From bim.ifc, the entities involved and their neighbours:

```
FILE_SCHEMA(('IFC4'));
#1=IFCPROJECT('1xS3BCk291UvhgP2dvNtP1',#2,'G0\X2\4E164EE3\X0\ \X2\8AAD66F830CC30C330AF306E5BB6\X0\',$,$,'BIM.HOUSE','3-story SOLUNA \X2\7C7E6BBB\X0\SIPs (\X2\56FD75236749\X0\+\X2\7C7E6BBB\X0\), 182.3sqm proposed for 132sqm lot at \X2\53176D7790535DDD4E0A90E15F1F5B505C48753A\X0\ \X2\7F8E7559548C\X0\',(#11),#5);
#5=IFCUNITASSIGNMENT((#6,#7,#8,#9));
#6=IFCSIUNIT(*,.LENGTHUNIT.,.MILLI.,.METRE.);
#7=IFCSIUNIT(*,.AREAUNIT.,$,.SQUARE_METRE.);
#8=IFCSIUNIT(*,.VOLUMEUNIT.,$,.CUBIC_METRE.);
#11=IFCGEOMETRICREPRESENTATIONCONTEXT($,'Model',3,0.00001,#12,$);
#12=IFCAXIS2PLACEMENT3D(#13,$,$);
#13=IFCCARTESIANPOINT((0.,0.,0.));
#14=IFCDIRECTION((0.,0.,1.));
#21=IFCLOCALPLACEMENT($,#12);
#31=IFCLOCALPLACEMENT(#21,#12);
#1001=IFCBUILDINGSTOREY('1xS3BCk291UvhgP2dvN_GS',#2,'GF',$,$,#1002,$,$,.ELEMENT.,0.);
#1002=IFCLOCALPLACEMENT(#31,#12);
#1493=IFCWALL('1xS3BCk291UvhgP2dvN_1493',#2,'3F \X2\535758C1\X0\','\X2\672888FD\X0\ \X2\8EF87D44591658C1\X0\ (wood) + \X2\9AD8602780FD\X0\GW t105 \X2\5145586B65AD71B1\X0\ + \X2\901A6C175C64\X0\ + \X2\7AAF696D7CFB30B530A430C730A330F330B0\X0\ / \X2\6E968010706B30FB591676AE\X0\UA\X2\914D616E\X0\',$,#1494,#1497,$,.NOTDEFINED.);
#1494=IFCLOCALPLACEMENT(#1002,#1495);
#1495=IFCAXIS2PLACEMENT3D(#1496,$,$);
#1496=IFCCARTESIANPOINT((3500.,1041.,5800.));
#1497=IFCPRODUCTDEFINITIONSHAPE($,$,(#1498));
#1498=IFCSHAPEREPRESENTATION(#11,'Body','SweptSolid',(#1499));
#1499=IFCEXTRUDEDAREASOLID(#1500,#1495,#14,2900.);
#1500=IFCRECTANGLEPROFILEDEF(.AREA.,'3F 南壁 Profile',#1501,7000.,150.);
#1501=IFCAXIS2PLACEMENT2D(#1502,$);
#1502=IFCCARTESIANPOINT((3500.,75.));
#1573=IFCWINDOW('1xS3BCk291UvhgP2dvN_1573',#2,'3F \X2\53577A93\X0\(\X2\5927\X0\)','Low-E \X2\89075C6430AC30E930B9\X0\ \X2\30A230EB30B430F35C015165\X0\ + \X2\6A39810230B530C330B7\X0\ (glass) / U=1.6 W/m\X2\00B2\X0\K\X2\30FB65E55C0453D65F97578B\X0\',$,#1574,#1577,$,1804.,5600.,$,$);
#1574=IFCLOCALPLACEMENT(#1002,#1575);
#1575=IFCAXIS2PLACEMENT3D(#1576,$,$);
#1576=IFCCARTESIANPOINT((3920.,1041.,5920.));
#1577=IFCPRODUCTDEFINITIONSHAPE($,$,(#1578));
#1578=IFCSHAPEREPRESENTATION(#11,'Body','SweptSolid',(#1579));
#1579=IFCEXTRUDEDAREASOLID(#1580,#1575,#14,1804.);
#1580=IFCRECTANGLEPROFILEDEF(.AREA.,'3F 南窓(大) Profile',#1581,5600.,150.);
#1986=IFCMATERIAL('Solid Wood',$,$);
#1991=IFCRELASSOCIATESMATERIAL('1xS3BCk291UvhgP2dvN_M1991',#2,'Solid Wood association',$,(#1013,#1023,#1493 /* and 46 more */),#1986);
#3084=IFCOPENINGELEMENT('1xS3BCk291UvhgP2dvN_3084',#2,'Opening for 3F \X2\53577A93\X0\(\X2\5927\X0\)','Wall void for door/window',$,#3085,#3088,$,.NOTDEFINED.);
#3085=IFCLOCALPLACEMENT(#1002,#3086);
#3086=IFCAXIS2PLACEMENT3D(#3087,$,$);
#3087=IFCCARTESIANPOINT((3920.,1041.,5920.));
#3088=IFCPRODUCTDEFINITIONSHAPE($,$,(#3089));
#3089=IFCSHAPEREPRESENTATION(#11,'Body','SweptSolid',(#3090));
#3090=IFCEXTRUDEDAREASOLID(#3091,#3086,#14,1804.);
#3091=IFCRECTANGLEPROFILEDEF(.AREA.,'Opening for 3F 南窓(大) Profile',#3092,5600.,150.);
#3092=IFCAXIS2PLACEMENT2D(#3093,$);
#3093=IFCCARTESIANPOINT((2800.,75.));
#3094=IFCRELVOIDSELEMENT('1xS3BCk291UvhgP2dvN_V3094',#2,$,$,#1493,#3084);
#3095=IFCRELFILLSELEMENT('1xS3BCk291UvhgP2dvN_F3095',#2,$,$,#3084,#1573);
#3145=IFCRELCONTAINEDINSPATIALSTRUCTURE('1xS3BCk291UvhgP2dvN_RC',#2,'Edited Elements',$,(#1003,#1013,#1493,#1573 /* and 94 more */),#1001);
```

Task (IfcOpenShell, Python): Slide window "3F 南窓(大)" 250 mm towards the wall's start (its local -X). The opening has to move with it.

```python
import ifcopenshell
import ifcopenshell.api.geometry
import ifcopenshell.util.placement

model = ifcopenshell.open("bim.ifc")

window = model.by_id(1573)
opening = window.FillsVoids[0].RelatingOpeningElement
wall = opening.VoidsElements[0].RelatingBuildingElement

wall_matrix = ifcopenshell.util.placement.get_local_placement(wall.ObjectPlacement)
shift = wall_matrix[:3, 0] * -250.0
before = ifcopenshell.util.placement.get_local_placement(window.ObjectPlacement)[:3, 3].copy()

# The window is not placed relative to its opening, so move both.
for product in (opening, window):
    matrix = ifcopenshell.util.placement.get_local_placement(product.ObjectPlacement)
    matrix[:3, 3] += shift
    ifcopenshell.api.geometry.edit_object_placement(model, product=product, matrix=matrix, is_si=False)

after = ifcopenshell.util.placement.get_local_placement(window.ObjectPlacement)[:3, 3]
print("window moved by", (after - before).round(3) + 0.0)

model.write("bim_edited.ifc")
```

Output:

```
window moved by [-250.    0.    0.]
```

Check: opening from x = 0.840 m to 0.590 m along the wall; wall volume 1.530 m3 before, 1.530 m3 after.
